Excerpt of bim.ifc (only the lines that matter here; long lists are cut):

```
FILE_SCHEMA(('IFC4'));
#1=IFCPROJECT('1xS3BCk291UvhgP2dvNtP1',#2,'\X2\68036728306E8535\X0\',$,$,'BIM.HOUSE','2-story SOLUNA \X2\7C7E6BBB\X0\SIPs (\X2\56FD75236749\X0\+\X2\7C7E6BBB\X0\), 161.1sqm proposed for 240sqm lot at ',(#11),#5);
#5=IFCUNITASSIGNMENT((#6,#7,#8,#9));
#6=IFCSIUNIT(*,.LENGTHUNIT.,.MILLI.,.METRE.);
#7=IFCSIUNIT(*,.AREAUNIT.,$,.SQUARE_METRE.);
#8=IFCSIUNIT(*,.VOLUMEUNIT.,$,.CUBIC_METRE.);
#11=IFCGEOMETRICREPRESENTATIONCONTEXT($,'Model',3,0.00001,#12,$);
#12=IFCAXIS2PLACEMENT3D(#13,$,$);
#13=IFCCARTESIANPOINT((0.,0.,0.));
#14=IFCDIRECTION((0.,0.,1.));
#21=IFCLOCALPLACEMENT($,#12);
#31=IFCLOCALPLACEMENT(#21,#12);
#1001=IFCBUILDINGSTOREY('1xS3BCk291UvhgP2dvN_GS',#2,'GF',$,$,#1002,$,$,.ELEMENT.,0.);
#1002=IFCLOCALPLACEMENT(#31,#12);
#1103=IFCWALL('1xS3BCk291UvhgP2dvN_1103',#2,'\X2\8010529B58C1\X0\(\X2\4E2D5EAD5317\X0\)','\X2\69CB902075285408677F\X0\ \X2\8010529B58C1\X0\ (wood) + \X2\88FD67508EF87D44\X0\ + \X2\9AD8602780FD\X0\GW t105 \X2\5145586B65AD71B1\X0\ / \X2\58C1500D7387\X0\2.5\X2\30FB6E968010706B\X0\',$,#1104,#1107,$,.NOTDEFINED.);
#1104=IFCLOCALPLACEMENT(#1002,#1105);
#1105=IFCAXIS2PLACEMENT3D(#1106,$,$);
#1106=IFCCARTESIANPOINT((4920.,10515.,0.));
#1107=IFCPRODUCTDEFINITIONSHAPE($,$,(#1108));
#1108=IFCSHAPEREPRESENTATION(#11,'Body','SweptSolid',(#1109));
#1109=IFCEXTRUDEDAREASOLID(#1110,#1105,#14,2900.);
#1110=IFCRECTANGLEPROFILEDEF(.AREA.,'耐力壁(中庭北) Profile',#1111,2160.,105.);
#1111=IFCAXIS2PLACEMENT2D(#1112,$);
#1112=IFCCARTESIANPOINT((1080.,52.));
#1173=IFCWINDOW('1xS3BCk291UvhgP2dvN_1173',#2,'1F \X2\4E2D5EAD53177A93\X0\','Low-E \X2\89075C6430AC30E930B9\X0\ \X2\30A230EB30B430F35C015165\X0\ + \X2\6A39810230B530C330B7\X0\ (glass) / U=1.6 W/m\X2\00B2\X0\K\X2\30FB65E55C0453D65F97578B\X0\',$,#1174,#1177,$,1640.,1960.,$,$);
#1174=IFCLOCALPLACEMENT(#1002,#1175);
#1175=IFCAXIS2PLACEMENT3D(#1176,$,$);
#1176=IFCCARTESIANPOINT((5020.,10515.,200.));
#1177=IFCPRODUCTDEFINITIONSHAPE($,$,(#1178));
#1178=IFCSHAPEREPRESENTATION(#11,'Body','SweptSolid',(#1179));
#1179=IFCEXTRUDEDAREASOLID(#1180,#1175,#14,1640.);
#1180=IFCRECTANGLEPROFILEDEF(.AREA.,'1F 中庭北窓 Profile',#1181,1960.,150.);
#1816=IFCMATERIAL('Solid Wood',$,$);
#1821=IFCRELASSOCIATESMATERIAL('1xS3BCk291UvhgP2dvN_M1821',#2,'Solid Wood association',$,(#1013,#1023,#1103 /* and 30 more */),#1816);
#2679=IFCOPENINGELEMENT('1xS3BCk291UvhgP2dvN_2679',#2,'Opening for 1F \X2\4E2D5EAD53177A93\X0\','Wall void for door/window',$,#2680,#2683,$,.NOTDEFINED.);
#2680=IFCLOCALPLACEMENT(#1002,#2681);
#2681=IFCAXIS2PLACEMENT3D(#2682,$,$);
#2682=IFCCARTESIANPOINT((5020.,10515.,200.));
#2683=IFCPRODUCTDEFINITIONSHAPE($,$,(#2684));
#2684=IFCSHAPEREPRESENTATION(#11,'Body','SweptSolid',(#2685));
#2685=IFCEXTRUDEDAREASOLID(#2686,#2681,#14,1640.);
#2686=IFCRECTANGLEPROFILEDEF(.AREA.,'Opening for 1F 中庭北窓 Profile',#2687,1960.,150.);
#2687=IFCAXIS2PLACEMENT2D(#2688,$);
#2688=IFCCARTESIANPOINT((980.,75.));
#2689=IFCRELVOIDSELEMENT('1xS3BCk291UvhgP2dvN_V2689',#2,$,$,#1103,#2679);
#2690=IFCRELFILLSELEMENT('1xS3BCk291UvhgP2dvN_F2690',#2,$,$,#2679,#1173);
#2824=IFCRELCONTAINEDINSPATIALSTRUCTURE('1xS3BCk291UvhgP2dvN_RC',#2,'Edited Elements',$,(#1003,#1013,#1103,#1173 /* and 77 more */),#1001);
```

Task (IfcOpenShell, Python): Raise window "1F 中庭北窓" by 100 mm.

```python
import numpy as np
import ifcopenshell
import ifcopenshell.api.geometry
import ifcopenshell.util.placement
import ifcopenshell.util.unit

model = ifcopenshell.open("bim.ifc")
unit_scale = ifcopenshell.util.unit.calculate_unit_scale(model)

window = model.by_guid("1xS3BCk291UvhgP2dvN_1173")
opening = window.FillsVoids[0].RelatingOpeningElement
dz = 0.1 / unit_scale

shift = np.array([0.0, 0.0, dz])
# The window is not placed relative to its opening, so move both.
for product in (opening, window):
    matrix = ifcopenshell.util.placement.get_local_placement(product.ObjectPlacement)
    matrix[:3, 3] += shift
    ifcopenshell.api.geometry.edit_object_placement(model, product=product, matrix=matrix, is_si=False)

print(f"moved by {dz * unit_scale:+.3f} m")

model.write("bim_updated.ifc")
```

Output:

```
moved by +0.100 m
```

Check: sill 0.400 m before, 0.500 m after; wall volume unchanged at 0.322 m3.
